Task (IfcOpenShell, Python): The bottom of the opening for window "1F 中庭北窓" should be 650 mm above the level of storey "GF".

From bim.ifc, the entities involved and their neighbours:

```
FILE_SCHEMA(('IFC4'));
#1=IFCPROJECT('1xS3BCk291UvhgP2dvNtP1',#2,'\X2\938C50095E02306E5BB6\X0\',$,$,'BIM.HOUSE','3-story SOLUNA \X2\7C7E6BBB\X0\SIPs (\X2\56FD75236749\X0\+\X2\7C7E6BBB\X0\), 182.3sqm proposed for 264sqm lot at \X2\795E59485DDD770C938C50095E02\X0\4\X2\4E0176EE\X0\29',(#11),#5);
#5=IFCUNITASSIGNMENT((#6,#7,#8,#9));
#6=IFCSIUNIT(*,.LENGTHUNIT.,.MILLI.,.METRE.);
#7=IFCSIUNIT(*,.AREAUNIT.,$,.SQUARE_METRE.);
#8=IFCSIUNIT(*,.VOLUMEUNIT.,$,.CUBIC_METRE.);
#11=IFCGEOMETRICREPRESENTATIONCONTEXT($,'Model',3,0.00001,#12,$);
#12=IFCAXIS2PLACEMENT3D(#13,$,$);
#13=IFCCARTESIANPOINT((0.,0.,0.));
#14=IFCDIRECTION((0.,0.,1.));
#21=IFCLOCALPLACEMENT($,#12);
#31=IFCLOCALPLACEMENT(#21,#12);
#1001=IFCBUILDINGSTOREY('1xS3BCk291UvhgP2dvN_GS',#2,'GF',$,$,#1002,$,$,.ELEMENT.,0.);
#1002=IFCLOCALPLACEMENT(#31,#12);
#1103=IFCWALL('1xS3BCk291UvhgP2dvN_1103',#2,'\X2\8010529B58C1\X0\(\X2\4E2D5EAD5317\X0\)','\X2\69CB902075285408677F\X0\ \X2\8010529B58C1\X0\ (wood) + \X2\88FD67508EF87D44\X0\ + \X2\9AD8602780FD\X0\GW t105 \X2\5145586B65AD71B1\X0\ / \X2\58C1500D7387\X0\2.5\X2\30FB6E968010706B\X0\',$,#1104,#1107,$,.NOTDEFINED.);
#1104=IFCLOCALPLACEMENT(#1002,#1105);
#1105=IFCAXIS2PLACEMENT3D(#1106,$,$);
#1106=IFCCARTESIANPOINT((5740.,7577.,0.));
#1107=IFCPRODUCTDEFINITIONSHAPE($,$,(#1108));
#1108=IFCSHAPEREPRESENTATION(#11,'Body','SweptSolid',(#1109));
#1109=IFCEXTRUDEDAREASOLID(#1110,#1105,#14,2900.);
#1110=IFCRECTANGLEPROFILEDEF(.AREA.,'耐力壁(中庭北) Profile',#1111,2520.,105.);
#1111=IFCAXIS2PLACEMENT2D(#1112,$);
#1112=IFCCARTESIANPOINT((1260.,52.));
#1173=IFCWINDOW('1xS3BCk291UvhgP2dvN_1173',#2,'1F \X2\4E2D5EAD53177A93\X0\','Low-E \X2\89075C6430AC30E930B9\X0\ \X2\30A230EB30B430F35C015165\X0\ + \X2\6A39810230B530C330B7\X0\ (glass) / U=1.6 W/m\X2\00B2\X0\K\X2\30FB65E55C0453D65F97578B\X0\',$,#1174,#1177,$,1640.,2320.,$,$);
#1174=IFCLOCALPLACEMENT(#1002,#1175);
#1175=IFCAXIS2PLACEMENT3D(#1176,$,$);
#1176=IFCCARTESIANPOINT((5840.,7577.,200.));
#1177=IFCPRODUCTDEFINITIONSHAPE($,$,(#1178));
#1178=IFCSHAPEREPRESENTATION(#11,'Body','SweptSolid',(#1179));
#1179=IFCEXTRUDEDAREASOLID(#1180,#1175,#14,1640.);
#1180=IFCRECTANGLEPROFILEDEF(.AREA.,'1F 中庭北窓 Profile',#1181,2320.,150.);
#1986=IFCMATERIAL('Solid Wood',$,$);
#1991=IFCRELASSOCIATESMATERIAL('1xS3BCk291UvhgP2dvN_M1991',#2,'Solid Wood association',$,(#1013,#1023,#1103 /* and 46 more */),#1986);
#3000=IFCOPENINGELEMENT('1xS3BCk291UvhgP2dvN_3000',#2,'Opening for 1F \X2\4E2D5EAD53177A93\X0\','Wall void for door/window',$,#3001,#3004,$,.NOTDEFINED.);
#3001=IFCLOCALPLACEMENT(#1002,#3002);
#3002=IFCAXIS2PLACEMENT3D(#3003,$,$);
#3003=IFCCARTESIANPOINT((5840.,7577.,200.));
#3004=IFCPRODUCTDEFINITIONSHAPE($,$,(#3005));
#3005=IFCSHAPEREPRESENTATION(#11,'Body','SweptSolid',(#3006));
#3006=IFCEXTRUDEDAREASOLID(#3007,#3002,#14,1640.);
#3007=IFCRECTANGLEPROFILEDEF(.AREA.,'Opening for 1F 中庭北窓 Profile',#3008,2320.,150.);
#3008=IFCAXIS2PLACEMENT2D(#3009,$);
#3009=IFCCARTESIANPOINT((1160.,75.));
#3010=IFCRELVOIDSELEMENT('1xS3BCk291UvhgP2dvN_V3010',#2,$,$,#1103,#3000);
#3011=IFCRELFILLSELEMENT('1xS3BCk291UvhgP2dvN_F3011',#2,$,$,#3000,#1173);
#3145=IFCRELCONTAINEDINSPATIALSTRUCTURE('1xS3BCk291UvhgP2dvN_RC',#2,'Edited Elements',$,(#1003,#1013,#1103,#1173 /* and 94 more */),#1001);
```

```python
import numpy as np
import ifcopenshell
import ifcopenshell.api.geometry
import ifcopenshell.geom
import ifcopenshell.util.element
import ifcopenshell.util.placement
import ifcopenshell.util.shape
import ifcopenshell.util.unit

model = ifcopenshell.open("bim.ifc")
unit_scale = ifcopenshell.util.unit.calculate_unit_scale(model)

window = model.by_id(1173)
opening = window.FillsVoids[0].RelatingOpeningElement
storey = ifcopenshell.util.element.get_container(window, ifc_class="IfcBuildingStorey")
level = ifcopenshell.util.placement.get_local_placement(storey.ObjectPlacement)[2, 3]

# The opening's origin need not be at the sill, so measure its lowest point.
shape = ifcopenshell.geom.create_shape(ifcopenshell.geom.settings(), opening)
bottom = ifcopenshell.util.shape.get_shape_bottom_elevation(shape, shape.geometry) / unit_scale
dz = level + 0.65 / unit_scale - bottom

shift = np.array([0.0, 0.0, dz])
# The window is not placed relative to its opening, so move both.
for product in (opening, window):
    matrix = ifcopenshell.util.placement.get_local_placement(product.ObjectPlacement)
    matrix[:3, 3] += shift
    ifcopenshell.api.geometry.edit_object_placement(model, product=product, matrix=matrix, is_si=False)

print(f"moved by {dz * unit_scale:+.3f} m")

model.write("bim_updated.ifc")
```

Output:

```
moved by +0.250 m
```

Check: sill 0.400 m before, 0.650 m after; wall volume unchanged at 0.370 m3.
